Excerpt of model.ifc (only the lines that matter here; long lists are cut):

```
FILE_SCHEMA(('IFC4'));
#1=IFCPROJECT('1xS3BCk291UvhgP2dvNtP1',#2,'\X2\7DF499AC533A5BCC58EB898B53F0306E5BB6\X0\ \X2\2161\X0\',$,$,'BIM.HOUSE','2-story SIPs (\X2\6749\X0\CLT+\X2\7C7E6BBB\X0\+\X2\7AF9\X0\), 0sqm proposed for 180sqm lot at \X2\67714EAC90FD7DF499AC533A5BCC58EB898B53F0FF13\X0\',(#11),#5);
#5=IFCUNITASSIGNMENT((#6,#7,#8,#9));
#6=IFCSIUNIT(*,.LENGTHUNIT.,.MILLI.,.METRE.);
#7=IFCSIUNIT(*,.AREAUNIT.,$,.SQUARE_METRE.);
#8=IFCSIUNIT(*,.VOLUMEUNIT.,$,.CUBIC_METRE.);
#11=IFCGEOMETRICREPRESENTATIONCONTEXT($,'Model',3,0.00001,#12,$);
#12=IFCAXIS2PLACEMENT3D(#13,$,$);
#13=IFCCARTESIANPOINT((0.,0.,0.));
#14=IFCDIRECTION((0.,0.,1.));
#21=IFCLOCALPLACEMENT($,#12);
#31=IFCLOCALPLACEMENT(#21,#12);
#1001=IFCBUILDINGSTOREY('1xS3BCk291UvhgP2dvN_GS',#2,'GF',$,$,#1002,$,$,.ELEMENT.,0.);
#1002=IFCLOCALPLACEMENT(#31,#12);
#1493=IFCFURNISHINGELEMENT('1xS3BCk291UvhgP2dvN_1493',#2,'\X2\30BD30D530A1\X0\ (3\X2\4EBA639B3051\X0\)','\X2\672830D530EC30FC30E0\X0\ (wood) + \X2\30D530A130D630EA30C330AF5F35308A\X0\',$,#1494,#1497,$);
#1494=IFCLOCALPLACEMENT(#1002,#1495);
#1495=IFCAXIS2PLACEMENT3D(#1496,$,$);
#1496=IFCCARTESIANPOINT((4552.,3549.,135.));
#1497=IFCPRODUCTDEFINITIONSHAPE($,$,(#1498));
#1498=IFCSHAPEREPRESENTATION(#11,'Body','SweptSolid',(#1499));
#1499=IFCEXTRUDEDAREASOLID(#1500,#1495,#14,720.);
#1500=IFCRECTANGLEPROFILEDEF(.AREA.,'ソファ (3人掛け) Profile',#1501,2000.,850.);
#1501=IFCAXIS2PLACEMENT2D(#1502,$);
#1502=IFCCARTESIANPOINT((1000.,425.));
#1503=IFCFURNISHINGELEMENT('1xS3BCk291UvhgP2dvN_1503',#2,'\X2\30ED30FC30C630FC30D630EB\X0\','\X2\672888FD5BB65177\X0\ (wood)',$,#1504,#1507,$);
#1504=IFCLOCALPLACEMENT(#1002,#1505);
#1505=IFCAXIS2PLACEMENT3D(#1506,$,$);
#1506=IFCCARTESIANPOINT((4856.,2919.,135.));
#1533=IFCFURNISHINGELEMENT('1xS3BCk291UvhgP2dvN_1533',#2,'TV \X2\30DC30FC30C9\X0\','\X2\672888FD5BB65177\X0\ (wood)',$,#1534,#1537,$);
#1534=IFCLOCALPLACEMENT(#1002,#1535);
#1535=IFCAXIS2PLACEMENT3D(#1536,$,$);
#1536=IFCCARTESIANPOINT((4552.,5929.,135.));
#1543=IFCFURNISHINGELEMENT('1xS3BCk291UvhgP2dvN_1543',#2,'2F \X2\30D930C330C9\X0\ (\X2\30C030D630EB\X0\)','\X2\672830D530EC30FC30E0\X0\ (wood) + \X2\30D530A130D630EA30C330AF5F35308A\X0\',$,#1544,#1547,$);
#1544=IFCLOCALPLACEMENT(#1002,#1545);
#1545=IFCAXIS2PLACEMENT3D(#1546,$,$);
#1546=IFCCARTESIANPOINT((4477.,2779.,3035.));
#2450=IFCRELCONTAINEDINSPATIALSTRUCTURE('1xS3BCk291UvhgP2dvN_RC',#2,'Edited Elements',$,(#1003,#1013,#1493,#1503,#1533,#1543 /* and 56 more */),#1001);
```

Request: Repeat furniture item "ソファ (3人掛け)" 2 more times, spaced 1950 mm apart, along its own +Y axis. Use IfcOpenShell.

```python
import ifcopenshell
import ifcopenshell.api.geometry
import ifcopenshell.api.root
import ifcopenshell.util.element
import ifcopenshell.util.placement

model = ifcopenshell.open("model.ifc")


def reuse_history(source, copy):
    """copy_class also copies each property set's owner history, people and application; keep the originals."""
    for rel in copy.IsDefinedBy:
        if rel.is_a("IfcRelDefinesByProperties") and (history := rel.RelatingPropertyDefinition.OwnerHistory):
            rel.RelatingPropertyDefinition.OwnerHistory = source.OwnerHistory
            ifcopenshell.util.element.remove_deep2(model, history)


source = model.by_guid("1xS3BCk291UvhgP2dvN_1493")
base = ifcopenshell.util.placement.get_local_placement(source.ObjectPlacement)
step = base[:3, 1] * 1950.0

for i in range(1, 3):
    copy = ifcopenshell.api.root.copy_class(model, product=source)
    copy.Representation = ifcopenshell.util.element.copy_deep(
        model, source.Representation, exclude=["IfcGeometricRepresentationContext", "IfcRepresentationMap"]
    )
    reuse_history(source, copy)
    matrix = base.copy()
    matrix[:3, 3] += i * step
    print("added at", matrix[:3, 3].round(3) + 0.0)
    ifcopenshell.api.geometry.edit_object_placement(model, product=copy, matrix=matrix, is_si=False)

model.write("model-out.ifc")
```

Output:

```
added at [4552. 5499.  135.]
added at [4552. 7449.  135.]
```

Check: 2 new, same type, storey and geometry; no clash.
